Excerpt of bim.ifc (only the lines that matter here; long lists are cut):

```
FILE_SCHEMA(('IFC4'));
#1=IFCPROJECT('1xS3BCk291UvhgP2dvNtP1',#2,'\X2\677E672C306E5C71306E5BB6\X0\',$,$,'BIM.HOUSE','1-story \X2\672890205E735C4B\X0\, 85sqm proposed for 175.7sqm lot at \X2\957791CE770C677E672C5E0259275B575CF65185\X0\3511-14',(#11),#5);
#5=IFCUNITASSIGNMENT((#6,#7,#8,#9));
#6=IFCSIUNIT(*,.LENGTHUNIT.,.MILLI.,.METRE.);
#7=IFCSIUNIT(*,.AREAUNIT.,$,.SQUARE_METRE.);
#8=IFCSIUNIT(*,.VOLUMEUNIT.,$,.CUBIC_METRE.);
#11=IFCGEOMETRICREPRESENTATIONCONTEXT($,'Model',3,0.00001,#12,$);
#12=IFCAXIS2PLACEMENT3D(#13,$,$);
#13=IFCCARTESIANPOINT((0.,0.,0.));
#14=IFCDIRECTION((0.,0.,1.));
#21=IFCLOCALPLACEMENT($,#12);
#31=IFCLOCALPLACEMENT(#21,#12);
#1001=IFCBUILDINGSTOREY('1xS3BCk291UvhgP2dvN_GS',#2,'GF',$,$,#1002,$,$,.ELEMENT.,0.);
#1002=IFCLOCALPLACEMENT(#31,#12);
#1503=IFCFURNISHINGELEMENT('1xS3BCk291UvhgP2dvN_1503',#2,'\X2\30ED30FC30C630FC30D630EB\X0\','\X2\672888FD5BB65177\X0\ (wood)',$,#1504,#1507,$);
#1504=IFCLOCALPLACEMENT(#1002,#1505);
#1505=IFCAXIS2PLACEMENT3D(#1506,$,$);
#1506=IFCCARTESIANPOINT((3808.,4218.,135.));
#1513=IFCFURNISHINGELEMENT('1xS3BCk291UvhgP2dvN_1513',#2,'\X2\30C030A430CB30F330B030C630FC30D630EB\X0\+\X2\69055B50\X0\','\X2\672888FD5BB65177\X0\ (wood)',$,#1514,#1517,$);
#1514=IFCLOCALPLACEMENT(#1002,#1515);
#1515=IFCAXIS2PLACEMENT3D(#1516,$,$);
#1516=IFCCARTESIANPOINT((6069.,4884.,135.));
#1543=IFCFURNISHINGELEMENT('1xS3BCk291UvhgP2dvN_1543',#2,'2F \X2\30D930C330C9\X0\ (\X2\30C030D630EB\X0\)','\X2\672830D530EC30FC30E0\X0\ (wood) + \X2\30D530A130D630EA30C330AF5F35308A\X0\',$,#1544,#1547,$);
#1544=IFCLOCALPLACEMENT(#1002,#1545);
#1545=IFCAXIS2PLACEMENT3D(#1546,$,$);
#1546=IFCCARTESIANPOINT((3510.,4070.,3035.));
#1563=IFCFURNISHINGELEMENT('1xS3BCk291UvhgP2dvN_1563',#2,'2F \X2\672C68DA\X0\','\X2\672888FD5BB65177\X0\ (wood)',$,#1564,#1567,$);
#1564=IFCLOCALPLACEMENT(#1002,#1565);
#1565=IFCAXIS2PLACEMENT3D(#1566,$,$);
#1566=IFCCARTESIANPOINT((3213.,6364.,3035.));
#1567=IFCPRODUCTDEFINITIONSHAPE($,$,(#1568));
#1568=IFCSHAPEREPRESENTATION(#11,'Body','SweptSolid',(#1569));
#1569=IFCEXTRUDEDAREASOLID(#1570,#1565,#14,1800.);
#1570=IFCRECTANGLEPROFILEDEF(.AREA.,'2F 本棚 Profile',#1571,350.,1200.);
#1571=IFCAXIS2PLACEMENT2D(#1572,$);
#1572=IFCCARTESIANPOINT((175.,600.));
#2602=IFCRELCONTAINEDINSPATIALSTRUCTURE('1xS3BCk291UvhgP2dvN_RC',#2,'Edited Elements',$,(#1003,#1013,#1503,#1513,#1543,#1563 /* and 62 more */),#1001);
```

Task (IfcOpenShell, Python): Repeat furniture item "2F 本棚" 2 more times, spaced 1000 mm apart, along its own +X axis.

```python
import ifcopenshell
import ifcopenshell.api.geometry
import ifcopenshell.api.root
import ifcopenshell.util.element
import ifcopenshell.util.placement
import ifcopenshell.util.unit

model = ifcopenshell.open("bim.ifc")
unit_scale = ifcopenshell.util.unit.calculate_unit_scale(model)


def reuse_history(source, copy):
    """copy_class also copies each property set's owner history, people and application; keep the originals."""
    for rel in copy.IsDefinedBy:
        if rel.is_a("IfcRelDefinesByProperties") and (history := rel.RelatingPropertyDefinition.OwnerHistory):
            rel.RelatingPropertyDefinition.OwnerHistory = source.OwnerHistory
            ifcopenshell.util.element.remove_deep2(model, history)


source = model.by_id(1563)
base = ifcopenshell.util.placement.get_local_placement(source.ObjectPlacement)
step = base[:3, 0] * 1 / unit_scale

for i in range(1, 3):
    copy = ifcopenshell.api.root.copy_class(model, product=source)
    copy.Representation = ifcopenshell.util.element.copy_deep(
        model, source.Representation, exclude=["IfcGeometricRepresentationContext", "IfcRepresentationMap"]
    )
    reuse_history(source, copy)
    matrix = base.copy()
    matrix[:3, 3] += i * step
    print("added at", matrix[:3, 3].round(3) + 0.0)
    ifcopenshell.api.geometry.edit_object_placement(model, product=copy, matrix=matrix, is_si=False)

model.write("bim-out.ifc")
```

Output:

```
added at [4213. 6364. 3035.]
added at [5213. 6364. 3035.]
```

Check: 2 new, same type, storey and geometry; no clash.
